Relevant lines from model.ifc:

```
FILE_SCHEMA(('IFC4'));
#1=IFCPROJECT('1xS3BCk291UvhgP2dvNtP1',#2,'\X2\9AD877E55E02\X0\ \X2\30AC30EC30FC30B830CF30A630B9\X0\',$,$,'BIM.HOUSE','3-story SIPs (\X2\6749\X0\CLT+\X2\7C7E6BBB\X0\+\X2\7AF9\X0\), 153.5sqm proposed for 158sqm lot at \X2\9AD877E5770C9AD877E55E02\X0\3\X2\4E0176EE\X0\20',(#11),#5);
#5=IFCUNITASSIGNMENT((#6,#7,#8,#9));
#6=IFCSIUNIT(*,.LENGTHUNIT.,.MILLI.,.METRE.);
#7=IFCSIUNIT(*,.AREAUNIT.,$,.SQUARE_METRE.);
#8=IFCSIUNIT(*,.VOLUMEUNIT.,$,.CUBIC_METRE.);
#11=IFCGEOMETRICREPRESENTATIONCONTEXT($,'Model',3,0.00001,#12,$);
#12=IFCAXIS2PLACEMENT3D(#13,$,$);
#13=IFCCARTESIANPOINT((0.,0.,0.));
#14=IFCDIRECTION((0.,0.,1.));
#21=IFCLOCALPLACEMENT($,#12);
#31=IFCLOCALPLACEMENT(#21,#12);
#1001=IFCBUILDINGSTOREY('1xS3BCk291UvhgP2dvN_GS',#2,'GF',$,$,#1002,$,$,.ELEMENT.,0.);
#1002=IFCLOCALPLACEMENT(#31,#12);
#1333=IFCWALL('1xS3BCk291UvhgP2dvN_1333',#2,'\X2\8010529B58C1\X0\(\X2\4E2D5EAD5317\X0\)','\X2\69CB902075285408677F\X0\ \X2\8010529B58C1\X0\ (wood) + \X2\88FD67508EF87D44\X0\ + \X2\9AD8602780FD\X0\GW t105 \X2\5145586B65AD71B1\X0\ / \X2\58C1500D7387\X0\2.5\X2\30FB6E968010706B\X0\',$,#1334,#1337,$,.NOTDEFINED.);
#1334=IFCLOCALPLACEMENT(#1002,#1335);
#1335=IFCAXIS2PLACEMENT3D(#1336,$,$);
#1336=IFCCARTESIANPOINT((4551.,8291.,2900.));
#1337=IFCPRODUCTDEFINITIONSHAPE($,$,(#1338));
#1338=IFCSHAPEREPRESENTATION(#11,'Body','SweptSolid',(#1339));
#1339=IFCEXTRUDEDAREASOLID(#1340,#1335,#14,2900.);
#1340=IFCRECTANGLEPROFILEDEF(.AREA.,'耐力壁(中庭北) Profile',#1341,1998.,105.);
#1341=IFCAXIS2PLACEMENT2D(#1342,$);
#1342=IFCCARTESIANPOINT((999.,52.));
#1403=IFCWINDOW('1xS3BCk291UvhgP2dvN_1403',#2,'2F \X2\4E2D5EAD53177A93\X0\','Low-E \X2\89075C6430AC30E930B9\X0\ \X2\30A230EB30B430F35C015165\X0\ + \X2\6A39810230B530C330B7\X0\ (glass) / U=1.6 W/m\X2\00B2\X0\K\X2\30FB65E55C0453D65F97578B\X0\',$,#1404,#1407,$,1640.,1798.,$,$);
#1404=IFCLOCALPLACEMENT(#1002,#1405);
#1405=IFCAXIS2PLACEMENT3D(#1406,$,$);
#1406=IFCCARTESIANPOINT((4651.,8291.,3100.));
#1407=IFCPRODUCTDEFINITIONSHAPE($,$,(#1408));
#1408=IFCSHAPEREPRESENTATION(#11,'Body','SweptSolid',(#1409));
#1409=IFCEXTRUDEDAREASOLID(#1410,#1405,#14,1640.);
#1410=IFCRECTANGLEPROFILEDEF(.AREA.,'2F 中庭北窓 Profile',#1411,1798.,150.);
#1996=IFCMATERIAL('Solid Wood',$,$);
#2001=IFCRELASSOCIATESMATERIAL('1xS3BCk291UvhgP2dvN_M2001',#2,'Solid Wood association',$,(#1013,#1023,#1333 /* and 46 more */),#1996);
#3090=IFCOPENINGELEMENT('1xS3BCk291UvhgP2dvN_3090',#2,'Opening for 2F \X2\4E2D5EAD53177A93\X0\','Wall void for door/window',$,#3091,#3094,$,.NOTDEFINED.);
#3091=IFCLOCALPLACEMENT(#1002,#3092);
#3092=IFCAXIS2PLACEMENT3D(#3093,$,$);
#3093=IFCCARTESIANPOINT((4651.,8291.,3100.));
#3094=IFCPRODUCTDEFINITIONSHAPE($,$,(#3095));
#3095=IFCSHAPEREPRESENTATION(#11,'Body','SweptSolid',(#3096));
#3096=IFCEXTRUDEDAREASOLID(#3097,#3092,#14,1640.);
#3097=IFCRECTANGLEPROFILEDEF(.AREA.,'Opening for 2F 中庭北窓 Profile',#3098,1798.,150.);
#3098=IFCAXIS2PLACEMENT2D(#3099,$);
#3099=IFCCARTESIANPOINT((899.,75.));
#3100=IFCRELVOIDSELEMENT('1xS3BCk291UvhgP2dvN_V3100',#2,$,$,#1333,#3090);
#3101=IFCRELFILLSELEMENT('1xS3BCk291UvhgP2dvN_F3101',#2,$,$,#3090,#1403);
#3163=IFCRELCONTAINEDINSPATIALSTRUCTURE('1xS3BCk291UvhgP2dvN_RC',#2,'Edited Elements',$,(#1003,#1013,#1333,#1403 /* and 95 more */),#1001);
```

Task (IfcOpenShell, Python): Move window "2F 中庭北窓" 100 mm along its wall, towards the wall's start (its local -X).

```python
import ifcopenshell
import ifcopenshell.api.geometry
import ifcopenshell.util.placement
import ifcopenshell.util.unit

model = ifcopenshell.open("model.ifc")
unit_scale = ifcopenshell.util.unit.calculate_unit_scale(model)

window = model.by_guid("1xS3BCk291UvhgP2dvN_1403")
opening = window.FillsVoids[0].RelatingOpeningElement
wall = opening.VoidsElements[0].RelatingBuildingElement

wall_matrix = ifcopenshell.util.placement.get_local_placement(wall.ObjectPlacement)
shift = wall_matrix[:3, 0] * -0.1 / unit_scale
before = ifcopenshell.util.placement.get_local_placement(window.ObjectPlacement)[:3, 3].copy()

# The window is not placed relative to its opening, so move both.
for product in (opening, window):
    matrix = ifcopenshell.util.placement.get_local_placement(product.ObjectPlacement)
    matrix[:3, 3] += shift
    ifcopenshell.api.geometry.edit_object_placement(model, product=product, matrix=matrix, is_si=False)

after = ifcopenshell.util.placement.get_local_placement(window.ObjectPlacement)[:3, 3]
print("window moved by", (after - before).round(3) + 0.0)

model.write("model_edited.ifc")
```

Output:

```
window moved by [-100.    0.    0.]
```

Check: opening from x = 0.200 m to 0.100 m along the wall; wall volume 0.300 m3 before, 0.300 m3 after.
